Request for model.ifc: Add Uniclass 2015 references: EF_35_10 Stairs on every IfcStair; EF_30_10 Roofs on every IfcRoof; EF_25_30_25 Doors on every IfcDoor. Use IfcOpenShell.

First a look at what the model holds.

```python
import ifcopenshell

model = ifcopenshell.open("model.ifc")
print(model.schema)
print("classifications:", [c.Name for c in model.by_type("IfcClassification")])
for ifc_class in ("IfcDoor", "IfcRoof", "IfcStair", "IfcWall", "IfcWindow"):
    print(ifc_class, len(model.by_type(ifc_class)))
```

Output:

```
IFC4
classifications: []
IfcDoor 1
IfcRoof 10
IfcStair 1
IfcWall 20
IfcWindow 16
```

```python
import ifcopenshell
import ifcopenshell.api.classification

model = ifcopenshell.open("model.ifc")

system = ifcopenshell.api.classification.add_classification(model, classification="Uniclass 2015")

codes = {
    "IfcStair": ("EF_35_10", "Stairs"),
    "IfcRoof": ("EF_30_10", "Roofs"),
    "IfcDoor": ("EF_25_30_25", "Doors"),
}
for ifc_class, (code, name) in codes.items():
    products = model.by_type(ifc_class)
    ifcopenshell.api.classification.add_reference(
        model, products=products, classification=system, identification=code, name=name
    )
    print(code, len(products))

model.write("model_rev.ifc")
```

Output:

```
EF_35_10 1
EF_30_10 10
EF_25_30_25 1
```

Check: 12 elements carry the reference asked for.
